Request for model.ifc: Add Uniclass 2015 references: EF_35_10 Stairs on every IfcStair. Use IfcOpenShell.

First a look at what the model holds.

```python
import ifcopenshell

model = ifcopenshell.open("model.ifc")
print(model.schema)
print("classifications:", [c.Name for c in model.by_type("IfcClassification")])
for ifc_class in ("IfcDoor", "IfcRoof", "IfcStair", "IfcWall", "IfcWindow"):
    print(ifc_class, len(model.by_type(ifc_class)))
```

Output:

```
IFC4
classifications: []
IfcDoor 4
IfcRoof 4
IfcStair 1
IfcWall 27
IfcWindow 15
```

```python
import ifcopenshell
import ifcopenshell.api.classification

model = ifcopenshell.open("model.ifc")

system = ifcopenshell.api.classification.add_classification(model, classification="Uniclass 2015")

codes = {
    "IfcStair": ("EF_35_10", "Stairs"),
}
for ifc_class, (code, name) in codes.items():
    products = model.by_type(ifc_class)
    ifcopenshell.api.classification.add_reference(
        model, products=products, classification=system, identification=code, name=name
    )
    print(code, len(products))

model.write("model_rev.ifc")
```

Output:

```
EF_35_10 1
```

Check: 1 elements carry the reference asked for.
